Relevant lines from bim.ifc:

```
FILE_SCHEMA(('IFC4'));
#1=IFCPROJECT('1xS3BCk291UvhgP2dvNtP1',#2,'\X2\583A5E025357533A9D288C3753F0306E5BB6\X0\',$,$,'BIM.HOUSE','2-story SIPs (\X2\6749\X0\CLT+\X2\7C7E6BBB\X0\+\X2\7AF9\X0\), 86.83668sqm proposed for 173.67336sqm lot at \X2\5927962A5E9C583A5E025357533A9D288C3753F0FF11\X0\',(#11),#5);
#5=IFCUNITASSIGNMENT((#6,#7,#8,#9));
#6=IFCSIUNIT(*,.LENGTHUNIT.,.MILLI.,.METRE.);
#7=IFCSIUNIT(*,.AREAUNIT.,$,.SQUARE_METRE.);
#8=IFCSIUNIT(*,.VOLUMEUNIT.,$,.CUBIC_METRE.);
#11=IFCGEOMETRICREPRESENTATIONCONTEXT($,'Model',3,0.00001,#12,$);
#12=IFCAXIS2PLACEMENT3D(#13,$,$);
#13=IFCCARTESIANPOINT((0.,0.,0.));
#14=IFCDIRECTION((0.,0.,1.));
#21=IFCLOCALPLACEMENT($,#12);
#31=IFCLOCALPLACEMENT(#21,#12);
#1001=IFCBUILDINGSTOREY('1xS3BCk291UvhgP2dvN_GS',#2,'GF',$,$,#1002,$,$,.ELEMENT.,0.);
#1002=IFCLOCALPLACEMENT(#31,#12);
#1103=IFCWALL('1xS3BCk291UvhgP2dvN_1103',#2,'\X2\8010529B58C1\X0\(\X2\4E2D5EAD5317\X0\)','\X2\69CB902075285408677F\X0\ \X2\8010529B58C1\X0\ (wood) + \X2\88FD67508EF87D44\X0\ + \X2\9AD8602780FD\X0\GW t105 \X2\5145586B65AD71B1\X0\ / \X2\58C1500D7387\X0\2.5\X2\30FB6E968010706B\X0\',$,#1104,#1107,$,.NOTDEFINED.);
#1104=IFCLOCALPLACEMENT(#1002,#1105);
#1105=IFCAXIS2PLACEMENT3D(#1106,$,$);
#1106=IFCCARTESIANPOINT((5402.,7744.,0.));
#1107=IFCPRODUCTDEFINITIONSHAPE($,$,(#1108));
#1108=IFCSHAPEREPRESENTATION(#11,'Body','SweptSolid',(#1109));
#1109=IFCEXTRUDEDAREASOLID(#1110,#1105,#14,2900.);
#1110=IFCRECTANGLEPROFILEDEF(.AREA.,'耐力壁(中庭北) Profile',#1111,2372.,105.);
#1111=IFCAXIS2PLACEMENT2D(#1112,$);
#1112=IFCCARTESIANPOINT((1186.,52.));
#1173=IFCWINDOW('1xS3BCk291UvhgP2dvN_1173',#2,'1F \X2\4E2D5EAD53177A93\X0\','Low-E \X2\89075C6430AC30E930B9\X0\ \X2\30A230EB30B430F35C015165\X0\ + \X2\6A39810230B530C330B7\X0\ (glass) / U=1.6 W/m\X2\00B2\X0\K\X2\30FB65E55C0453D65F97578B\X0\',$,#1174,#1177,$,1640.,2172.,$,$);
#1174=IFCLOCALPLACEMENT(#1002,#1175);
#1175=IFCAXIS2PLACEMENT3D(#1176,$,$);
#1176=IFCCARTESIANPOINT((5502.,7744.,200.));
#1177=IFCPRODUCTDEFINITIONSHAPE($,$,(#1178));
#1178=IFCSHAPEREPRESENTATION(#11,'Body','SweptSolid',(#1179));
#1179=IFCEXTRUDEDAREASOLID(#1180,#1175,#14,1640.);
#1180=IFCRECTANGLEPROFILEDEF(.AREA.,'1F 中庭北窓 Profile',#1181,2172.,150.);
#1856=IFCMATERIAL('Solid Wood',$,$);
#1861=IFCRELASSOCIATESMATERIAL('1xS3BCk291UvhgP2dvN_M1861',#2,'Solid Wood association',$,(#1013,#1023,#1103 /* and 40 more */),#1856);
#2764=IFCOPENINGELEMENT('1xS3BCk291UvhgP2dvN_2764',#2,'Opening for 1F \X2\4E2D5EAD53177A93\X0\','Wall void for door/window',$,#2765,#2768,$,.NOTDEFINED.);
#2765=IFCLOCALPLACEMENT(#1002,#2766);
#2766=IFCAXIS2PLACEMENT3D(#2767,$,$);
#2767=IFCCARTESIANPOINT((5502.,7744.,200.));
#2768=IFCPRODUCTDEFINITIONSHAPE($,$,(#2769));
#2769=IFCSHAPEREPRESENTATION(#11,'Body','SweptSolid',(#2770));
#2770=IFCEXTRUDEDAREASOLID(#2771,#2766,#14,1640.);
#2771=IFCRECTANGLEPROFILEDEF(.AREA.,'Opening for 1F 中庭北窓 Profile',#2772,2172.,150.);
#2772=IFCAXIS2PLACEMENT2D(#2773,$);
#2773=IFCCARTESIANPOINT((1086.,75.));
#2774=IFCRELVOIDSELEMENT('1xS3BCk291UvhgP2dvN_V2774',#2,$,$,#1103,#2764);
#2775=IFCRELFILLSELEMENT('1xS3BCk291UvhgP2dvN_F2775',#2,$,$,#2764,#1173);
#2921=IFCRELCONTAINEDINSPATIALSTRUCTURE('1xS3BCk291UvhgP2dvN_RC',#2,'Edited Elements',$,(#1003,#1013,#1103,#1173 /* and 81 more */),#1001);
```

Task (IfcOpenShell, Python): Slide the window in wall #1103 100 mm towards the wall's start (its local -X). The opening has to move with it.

```python
import ifcopenshell
import ifcopenshell.api.geometry
import ifcopenshell.util.placement
import ifcopenshell.util.unit

model = ifcopenshell.open("bim.ifc")
unit_scale = ifcopenshell.util.unit.calculate_unit_scale(model)

window = model.by_guid("1xS3BCk291UvhgP2dvN_1173")
opening = window.FillsVoids[0].RelatingOpeningElement
wall = opening.VoidsElements[0].RelatingBuildingElement

wall_matrix = ifcopenshell.util.placement.get_local_placement(wall.ObjectPlacement)
shift = wall_matrix[:3, 0] * -0.1 / unit_scale
before = ifcopenshell.util.placement.get_local_placement(window.ObjectPlacement)[:3, 3].copy()

# The window is not placed relative to its opening, so move both.
for product in (opening, window):
    matrix = ifcopenshell.util.placement.get_local_placement(product.ObjectPlacement)
    matrix[:3, 3] += shift
    ifcopenshell.api.geometry.edit_object_placement(model, product=product, matrix=matrix, is_si=False)

after = ifcopenshell.util.placement.get_local_placement(window.ObjectPlacement)[:3, 3]
print("window moved by", (after - before).round(3) + 0.0)

model.write("bim_edited.ifc")
```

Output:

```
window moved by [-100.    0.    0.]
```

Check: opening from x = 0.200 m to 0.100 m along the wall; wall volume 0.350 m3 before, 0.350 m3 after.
